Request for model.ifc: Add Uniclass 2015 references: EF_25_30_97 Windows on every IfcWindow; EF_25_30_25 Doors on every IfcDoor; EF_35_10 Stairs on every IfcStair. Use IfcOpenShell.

First a look at what the model holds.

```python
import ifcopenshell

model = ifcopenshell.open("model.ifc")
print(model.schema)
print("classifications:", [c.Name for c in model.by_type("IfcClassification")])
for ifc_class in ("IfcDoor", "IfcRoof", "IfcStair", "IfcWall", "IfcWindow"):
    print(ifc_class, len(model.by_type(ifc_class)))
```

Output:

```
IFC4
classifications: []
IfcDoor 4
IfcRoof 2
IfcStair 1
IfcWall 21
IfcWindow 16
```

```python
import ifcopenshell
import ifcopenshell.api.classification

model = ifcopenshell.open("model.ifc")

system = ifcopenshell.api.classification.add_classification(model, classification="Uniclass 2015")

codes = {
    "IfcWindow": ("EF_25_30_97", "Windows"),
    "IfcDoor": ("EF_25_30_25", "Doors"),
    "IfcStair": ("EF_35_10", "Stairs"),
}
for ifc_class, (code, name) in codes.items():
    products = model.by_type(ifc_class)
    ifcopenshell.api.classification.add_reference(
        model, products=products, classification=system, identification=code, name=name
    )
    print(code, len(products))

model.write("model_v2.ifc")
```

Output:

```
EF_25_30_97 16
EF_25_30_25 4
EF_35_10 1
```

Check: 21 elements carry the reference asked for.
